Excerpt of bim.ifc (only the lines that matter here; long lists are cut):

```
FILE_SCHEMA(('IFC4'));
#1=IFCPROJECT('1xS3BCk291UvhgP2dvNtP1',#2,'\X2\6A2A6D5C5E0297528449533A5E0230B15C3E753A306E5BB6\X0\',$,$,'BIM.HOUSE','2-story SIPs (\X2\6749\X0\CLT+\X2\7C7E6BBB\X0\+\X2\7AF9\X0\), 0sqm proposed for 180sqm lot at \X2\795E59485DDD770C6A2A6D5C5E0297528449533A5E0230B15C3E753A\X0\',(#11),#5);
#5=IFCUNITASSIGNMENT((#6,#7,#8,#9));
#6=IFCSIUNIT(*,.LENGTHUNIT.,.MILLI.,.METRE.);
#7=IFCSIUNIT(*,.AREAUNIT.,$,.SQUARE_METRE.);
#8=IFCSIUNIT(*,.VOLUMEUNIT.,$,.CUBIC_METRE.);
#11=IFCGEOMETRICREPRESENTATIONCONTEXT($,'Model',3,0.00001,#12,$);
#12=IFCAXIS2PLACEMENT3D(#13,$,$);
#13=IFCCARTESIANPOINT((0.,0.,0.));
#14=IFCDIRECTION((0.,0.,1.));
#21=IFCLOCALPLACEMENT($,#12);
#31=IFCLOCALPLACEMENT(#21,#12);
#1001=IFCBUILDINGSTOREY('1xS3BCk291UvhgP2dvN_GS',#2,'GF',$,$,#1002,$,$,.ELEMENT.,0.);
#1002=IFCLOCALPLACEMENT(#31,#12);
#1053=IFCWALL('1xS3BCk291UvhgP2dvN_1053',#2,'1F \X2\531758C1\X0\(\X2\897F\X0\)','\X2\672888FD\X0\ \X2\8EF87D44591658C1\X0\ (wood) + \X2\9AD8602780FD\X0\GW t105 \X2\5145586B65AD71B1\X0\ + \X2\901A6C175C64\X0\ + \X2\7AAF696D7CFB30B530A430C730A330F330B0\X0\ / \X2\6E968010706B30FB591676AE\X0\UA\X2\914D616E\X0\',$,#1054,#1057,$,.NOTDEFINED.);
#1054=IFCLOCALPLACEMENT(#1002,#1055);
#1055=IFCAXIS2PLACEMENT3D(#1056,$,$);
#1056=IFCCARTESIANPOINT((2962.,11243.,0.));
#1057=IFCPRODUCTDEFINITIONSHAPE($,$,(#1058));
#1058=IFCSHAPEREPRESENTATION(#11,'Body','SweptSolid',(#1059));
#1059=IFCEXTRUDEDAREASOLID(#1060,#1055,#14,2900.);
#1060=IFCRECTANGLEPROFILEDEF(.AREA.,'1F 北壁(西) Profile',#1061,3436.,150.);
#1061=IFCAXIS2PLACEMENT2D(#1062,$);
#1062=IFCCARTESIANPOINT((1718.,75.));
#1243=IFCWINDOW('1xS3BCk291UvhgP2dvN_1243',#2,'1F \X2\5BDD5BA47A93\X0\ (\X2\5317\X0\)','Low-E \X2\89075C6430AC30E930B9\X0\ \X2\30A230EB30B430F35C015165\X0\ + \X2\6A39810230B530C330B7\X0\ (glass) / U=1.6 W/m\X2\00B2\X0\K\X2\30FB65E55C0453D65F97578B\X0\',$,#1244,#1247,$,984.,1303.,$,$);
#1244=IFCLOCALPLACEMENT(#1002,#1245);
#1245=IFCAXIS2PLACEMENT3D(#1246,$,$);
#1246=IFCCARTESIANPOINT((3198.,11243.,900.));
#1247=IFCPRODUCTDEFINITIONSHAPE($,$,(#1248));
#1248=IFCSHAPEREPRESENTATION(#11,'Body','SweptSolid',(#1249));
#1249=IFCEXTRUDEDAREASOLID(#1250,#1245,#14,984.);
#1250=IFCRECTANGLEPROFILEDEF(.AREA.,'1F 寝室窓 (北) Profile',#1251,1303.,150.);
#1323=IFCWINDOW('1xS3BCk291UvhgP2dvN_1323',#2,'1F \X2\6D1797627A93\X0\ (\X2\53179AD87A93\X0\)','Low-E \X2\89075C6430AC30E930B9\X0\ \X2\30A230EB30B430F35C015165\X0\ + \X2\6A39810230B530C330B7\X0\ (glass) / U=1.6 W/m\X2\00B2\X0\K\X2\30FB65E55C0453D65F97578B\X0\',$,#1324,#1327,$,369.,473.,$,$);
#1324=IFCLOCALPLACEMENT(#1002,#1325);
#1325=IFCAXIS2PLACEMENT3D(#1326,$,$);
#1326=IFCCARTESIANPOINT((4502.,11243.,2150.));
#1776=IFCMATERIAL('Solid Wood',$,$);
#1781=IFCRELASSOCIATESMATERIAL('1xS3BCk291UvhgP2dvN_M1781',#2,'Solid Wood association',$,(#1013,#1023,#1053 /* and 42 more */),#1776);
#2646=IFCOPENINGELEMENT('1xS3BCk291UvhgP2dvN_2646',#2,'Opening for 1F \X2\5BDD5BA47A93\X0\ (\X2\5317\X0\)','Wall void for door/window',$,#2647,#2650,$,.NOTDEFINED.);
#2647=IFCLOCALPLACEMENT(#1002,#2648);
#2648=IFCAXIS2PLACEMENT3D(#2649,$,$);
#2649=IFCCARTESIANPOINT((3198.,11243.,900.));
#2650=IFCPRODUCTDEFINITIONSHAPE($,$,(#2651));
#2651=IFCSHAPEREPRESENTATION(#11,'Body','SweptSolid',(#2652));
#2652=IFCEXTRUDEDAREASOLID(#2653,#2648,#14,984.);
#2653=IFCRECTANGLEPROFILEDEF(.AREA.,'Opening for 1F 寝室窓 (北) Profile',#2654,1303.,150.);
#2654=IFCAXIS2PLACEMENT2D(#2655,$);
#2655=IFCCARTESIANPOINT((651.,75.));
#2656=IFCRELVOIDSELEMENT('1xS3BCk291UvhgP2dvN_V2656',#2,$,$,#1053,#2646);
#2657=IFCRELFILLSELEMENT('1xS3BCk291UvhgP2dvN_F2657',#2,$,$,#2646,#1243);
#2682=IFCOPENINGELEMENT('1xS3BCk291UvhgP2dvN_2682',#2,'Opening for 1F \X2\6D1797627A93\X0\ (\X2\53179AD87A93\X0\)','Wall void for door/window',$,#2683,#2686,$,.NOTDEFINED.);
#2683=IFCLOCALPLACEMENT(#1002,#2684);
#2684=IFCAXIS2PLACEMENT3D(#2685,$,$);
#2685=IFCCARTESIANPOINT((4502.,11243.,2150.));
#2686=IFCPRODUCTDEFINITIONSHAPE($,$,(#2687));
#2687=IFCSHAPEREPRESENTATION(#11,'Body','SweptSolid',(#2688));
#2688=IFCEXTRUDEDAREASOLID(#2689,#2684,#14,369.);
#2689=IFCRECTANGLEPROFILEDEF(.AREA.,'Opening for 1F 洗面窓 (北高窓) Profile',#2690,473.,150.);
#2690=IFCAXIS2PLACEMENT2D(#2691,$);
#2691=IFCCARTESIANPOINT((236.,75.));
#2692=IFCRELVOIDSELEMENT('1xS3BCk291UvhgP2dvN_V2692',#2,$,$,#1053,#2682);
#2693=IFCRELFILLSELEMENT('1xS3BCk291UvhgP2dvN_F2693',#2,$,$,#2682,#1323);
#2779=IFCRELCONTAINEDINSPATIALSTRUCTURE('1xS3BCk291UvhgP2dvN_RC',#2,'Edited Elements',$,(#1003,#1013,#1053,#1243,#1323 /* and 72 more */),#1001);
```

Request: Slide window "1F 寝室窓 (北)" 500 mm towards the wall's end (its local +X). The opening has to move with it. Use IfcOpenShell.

```python
import ifcopenshell
import ifcopenshell.api.geometry
import ifcopenshell.util.placement

model = ifcopenshell.open("bim.ifc")

window = model.by_guid("1xS3BCk291UvhgP2dvN_1243")
opening = window.FillsVoids[0].RelatingOpeningElement
wall = opening.VoidsElements[0].RelatingBuildingElement

wall_matrix = ifcopenshell.util.placement.get_local_placement(wall.ObjectPlacement)
shift = wall_matrix[:3, 0] * 500.0
before = ifcopenshell.util.placement.get_local_placement(window.ObjectPlacement)[:3, 3].copy()

# The window is not placed relative to its opening, so move both.
for product in (opening, window):
    matrix = ifcopenshell.util.placement.get_local_placement(product.ObjectPlacement)
    matrix[:3, 3] += shift
    ifcopenshell.api.geometry.edit_object_placement(model, product=product, matrix=matrix, is_si=False)

after = ifcopenshell.util.placement.get_local_placement(window.ObjectPlacement)[:3, 3]
print("window moved by", (after - before).round(3) + 0.0)

model.write("bim_rev.ifc")
```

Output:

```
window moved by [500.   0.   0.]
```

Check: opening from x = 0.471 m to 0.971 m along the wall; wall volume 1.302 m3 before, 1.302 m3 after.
